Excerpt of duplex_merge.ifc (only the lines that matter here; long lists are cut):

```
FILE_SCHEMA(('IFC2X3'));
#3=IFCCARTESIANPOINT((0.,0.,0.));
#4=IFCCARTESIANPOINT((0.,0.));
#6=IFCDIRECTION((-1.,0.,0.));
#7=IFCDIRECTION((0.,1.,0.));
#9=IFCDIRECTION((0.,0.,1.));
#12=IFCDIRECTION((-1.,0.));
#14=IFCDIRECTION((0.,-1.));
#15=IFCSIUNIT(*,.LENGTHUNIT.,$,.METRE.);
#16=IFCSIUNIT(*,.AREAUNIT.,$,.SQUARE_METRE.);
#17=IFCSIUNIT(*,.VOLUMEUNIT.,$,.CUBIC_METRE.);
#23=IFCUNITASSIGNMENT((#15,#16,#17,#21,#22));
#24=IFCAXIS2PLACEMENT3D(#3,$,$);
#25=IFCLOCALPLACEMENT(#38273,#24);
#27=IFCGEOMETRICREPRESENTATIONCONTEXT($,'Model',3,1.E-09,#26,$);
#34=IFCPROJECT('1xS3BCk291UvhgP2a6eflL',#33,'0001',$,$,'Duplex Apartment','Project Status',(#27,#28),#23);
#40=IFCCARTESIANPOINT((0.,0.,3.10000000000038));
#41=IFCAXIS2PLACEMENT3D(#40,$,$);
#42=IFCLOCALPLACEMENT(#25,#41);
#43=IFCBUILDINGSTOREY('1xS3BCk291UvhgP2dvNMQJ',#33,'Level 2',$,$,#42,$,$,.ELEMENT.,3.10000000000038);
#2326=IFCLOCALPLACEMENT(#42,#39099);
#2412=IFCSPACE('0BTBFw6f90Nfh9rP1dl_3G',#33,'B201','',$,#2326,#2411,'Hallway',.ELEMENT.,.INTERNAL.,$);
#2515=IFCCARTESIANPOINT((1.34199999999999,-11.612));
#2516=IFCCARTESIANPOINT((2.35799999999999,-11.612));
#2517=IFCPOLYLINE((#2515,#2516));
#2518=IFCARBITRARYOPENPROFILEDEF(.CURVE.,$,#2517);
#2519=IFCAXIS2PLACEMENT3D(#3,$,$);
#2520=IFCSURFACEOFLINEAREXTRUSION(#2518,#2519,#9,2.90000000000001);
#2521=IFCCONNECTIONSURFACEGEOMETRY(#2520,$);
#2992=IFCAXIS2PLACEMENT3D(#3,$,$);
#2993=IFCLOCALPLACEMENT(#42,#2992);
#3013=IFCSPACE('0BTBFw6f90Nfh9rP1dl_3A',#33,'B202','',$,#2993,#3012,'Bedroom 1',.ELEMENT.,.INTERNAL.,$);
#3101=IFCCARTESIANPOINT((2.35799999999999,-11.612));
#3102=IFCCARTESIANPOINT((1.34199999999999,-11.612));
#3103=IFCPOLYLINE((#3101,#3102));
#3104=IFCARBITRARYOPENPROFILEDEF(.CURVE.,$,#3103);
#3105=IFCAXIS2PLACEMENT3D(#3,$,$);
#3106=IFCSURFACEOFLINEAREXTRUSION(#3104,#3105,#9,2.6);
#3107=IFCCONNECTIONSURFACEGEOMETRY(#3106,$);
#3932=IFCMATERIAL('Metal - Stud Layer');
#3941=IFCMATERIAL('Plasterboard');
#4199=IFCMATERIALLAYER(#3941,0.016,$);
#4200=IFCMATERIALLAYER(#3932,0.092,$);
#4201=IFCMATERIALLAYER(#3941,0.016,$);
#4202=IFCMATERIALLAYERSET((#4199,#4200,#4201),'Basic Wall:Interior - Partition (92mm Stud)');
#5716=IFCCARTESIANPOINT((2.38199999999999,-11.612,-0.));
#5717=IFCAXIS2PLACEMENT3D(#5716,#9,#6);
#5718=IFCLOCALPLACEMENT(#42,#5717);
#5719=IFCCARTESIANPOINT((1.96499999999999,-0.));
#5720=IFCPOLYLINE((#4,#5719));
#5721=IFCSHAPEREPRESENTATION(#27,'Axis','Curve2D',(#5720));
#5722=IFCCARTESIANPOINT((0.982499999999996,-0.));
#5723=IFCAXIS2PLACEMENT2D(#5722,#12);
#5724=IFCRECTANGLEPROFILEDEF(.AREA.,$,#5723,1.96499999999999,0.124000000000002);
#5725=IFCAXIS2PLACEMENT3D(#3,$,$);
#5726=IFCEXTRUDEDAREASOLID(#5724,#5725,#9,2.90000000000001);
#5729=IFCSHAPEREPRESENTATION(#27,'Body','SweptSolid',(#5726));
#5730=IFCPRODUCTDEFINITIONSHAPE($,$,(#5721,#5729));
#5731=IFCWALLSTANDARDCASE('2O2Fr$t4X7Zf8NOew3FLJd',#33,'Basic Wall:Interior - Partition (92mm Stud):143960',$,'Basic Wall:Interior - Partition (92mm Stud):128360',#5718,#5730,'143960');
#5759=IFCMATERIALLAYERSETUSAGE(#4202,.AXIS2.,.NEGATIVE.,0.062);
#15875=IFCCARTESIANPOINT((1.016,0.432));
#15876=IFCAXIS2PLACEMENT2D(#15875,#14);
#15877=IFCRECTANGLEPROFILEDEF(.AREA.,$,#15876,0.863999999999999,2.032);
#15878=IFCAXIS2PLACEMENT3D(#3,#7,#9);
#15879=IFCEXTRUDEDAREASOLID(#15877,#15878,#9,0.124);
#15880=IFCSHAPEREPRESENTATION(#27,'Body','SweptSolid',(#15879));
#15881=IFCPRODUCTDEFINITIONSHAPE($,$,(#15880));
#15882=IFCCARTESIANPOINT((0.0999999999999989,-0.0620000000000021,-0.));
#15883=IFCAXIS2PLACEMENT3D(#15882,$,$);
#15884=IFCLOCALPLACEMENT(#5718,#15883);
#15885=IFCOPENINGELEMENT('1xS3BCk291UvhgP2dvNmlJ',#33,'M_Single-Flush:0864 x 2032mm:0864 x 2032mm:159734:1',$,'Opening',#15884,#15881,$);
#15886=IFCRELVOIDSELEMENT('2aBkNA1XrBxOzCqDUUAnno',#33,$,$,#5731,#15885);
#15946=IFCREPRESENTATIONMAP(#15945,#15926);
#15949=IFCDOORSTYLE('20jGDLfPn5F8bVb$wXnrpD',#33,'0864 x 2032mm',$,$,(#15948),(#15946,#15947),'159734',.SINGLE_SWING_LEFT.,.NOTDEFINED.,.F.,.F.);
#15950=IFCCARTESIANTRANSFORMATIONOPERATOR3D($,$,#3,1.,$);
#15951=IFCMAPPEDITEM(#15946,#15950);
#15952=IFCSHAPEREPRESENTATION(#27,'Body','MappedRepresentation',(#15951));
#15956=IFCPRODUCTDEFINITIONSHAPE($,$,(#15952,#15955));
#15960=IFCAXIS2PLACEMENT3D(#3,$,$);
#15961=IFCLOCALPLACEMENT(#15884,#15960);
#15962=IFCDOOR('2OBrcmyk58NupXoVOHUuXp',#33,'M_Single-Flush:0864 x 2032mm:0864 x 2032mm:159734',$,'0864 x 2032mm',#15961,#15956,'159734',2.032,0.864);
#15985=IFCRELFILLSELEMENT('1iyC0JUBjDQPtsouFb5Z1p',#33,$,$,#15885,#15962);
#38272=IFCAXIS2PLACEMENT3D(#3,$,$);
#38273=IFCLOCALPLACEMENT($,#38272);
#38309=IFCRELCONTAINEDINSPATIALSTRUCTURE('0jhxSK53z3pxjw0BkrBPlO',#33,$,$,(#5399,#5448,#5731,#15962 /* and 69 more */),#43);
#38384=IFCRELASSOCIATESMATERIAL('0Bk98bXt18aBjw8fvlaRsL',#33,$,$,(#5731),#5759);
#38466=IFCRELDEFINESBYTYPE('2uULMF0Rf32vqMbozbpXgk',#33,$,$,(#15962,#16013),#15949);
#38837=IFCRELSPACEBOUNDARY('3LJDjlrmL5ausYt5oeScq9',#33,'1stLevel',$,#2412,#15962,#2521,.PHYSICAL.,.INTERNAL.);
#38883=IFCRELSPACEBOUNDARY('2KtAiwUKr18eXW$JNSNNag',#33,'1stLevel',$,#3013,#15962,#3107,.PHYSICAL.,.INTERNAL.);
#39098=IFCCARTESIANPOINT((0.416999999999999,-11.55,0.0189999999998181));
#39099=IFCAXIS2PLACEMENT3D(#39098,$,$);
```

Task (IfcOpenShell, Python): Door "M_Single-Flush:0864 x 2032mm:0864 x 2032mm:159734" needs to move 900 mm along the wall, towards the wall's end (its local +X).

```python
import numpy as np
import ifcopenshell
import ifcopenshell.api.geometry
import ifcopenshell.util.placement
import ifcopenshell.util.unit

model = ifcopenshell.open("duplex_merge.ifc")
unit_scale = ifcopenshell.util.unit.calculate_unit_scale(model)

door = model.by_guid("2OBrcmyk58NupXoVOHUuXp")
opening = door.FillsVoids[0].RelatingOpeningElement
wall = opening.VoidsElements[0].RelatingBuildingElement

wall_matrix = ifcopenshell.util.placement.get_local_placement(wall.ObjectPlacement)
shift = wall_matrix[:3, 0] * 0.9 / unit_scale
before = ifcopenshell.util.placement.get_local_placement(door.ObjectPlacement)[:3, 3].copy()

# The door is placed relative to its opening, so it follows when the opening moves.
matrix = ifcopenshell.util.placement.get_local_placement(opening.ObjectPlacement)
matrix[:3, 3] += shift
ifcopenshell.api.geometry.edit_object_placement(
    model, product=opening, matrix=matrix, is_si=False, should_transform_children=True
)

# Space boundary surfaces are stored in each space's coordinates; move them too.
for rel in door.ProvidesBoundaries:
    if not rel.ConnectionGeometry:
        continue
    surface = rel.ConnectionGeometry.SurfaceOnRelatingElement
    space_matrix = ifcopenshell.util.placement.get_local_placement(rel.RelatingSpace.ObjectPlacement)
    point = np.array(surface.Position.Location.Coordinates) + space_matrix[:3, :3].T @ shift
    surface.Position = model.createIfcAxis2Placement3D(
        model.createIfcCartesianPoint(point.tolist()), surface.Position.Axis, surface.Position.RefDirection
    )

after = ifcopenshell.util.placement.get_local_placement(door.ObjectPlacement)[:3, 3]
print("door moved by", (after - before).round(3) + 0.0)

model.write("duplex_merge_edited.ifc")
```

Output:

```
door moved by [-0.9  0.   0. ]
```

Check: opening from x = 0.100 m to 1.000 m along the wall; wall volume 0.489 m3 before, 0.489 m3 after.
